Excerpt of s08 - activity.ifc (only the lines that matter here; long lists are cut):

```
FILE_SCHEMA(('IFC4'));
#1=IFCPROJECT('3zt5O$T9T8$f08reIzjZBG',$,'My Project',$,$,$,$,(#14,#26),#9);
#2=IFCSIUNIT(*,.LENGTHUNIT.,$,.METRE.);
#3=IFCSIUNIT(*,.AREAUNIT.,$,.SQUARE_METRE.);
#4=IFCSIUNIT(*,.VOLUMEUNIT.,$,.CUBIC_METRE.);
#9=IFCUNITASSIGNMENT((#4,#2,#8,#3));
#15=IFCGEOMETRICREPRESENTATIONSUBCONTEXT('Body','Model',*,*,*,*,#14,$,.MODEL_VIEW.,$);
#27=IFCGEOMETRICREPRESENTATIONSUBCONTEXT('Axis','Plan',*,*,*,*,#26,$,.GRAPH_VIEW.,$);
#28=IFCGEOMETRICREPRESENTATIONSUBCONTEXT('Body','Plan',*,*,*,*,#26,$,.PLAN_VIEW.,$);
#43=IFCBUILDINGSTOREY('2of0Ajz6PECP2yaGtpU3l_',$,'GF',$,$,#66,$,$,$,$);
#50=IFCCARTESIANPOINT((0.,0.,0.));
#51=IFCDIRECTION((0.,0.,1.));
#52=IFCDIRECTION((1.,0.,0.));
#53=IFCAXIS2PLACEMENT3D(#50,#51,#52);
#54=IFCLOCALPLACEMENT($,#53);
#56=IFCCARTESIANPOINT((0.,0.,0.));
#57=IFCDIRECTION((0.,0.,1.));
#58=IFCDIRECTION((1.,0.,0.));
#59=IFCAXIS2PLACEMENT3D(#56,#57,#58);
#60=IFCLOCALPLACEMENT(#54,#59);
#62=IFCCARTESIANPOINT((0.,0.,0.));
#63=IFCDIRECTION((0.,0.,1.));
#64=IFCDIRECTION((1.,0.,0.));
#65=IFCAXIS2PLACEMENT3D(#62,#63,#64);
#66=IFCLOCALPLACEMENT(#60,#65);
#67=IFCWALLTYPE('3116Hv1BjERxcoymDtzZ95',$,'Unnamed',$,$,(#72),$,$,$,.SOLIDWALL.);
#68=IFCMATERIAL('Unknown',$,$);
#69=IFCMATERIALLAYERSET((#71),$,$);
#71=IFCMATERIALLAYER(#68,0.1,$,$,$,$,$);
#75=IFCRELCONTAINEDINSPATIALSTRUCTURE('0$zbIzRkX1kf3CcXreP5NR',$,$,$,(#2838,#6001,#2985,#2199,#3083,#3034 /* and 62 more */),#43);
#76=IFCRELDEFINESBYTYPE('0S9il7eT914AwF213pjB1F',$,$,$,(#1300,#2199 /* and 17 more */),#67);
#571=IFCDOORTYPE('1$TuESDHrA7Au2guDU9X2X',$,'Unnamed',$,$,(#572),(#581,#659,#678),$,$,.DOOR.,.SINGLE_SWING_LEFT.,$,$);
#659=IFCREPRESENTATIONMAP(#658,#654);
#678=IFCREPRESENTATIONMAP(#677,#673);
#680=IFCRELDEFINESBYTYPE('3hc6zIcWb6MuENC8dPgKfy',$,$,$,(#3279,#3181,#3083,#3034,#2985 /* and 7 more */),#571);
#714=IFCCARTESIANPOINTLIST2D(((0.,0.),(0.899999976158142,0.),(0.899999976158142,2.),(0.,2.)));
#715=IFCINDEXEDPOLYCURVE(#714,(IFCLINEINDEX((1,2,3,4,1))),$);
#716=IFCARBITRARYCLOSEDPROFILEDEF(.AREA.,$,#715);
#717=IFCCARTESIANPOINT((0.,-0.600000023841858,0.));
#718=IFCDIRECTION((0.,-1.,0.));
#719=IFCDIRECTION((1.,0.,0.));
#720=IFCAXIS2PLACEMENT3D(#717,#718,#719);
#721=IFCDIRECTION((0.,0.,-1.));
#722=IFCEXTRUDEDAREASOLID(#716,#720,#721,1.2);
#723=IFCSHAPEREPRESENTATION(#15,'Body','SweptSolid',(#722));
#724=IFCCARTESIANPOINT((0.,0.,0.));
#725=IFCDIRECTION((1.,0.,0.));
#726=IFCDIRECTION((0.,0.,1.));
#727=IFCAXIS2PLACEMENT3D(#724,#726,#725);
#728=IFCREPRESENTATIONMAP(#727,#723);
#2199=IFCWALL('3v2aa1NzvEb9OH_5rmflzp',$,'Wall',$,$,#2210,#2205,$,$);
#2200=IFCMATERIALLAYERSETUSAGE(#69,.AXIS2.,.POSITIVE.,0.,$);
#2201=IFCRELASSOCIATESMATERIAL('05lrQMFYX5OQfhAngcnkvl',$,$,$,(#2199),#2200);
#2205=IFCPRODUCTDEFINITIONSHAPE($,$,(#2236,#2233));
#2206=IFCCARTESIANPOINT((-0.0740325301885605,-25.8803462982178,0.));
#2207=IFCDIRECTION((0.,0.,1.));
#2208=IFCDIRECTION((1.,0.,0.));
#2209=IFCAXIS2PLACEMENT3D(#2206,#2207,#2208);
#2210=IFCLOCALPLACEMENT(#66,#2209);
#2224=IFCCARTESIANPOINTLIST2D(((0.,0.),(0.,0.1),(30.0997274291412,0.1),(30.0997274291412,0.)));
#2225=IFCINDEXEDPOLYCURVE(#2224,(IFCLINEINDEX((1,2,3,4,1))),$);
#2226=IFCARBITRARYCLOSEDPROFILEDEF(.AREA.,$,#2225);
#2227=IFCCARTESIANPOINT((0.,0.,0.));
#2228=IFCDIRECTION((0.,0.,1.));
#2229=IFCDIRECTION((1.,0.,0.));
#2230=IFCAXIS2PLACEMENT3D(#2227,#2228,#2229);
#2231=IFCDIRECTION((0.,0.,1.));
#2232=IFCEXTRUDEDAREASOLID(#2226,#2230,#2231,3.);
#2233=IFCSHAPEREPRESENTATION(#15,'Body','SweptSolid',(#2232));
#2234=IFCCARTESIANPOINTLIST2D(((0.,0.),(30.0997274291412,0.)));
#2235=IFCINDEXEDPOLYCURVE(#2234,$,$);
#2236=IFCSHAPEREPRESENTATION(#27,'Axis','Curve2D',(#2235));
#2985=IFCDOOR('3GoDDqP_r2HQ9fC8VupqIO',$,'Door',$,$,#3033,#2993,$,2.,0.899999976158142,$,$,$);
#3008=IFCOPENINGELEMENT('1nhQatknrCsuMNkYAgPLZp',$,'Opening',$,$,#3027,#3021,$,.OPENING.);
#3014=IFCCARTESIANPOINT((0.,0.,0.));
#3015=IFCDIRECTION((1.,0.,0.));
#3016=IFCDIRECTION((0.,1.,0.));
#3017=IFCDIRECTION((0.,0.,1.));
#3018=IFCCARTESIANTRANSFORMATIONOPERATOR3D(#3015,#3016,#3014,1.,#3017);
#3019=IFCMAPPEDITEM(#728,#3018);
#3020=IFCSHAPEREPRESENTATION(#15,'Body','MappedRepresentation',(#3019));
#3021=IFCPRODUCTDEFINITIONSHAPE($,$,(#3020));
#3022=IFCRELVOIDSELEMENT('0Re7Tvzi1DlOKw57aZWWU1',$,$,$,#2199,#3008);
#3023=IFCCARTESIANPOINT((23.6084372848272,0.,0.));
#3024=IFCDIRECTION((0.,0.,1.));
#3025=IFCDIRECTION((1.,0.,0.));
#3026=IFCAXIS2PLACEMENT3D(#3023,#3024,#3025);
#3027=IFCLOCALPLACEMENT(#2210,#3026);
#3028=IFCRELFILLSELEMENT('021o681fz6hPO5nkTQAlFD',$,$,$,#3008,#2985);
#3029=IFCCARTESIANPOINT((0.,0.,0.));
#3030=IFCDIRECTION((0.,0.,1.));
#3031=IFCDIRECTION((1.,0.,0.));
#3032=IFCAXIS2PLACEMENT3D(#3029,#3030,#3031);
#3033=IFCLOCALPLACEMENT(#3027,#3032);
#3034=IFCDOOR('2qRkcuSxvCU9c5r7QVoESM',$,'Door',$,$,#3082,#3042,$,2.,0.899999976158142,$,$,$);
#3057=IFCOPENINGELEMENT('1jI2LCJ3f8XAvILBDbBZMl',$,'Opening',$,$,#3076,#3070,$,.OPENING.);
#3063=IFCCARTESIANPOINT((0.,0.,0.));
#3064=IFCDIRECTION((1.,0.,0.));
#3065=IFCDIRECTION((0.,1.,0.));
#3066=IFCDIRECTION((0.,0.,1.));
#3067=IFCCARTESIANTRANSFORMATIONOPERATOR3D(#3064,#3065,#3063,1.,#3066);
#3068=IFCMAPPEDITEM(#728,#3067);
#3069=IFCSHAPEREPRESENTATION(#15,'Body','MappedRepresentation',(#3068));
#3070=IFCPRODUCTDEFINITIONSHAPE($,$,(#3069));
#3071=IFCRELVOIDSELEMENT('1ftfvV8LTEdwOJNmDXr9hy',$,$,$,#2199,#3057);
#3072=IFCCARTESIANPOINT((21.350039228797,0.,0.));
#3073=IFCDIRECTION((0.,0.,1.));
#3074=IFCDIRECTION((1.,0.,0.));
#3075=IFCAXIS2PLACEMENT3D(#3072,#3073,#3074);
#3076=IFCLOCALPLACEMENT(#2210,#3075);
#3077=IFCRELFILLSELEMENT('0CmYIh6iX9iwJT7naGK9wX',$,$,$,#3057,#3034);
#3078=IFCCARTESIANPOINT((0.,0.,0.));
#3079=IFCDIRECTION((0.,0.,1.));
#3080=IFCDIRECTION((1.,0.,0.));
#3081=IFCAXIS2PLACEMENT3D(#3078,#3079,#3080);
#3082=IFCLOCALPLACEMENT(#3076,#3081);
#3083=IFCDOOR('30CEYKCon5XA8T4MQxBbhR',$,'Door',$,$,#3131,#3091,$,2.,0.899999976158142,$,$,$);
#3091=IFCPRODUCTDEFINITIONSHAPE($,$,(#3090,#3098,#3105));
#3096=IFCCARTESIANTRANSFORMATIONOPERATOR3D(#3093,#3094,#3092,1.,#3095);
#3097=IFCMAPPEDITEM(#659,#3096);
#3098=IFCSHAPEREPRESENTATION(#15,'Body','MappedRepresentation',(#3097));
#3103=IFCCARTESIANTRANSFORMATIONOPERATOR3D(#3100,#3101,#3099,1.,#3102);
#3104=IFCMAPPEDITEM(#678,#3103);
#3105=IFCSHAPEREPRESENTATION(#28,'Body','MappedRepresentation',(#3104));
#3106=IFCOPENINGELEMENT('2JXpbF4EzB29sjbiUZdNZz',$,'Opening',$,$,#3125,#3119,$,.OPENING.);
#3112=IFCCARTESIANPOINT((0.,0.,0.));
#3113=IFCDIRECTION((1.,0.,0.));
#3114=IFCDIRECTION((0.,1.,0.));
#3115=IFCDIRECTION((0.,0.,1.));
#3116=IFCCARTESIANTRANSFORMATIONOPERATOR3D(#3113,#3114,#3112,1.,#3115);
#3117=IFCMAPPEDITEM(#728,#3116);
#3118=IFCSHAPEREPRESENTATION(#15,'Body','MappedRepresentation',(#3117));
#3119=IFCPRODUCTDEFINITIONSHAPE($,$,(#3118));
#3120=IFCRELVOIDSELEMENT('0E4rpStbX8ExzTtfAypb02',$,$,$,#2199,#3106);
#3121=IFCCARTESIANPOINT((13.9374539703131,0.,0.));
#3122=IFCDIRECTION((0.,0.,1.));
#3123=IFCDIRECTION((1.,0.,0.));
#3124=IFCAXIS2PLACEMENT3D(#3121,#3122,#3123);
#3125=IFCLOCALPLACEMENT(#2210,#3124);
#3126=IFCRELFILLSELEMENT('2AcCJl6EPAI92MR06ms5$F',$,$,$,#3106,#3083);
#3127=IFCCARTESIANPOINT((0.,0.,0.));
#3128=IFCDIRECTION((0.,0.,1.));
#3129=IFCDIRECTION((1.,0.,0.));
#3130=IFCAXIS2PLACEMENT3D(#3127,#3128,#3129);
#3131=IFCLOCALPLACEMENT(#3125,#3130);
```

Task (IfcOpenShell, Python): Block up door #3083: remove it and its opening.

```python
import ifcopenshell
import ifcopenshell.api.feature
import ifcopenshell.api.root
import ifcopenshell.geom
import ifcopenshell.util.shape

model = ifcopenshell.open("s08 - activity.ifc")
settings = ifcopenshell.geom.settings()


def volume(element):
    """Net volume in cubic metres, openings subtracted."""
    shape = ifcopenshell.geom.create_shape(settings, element)
    return ifcopenshell.util.shape.get_volume(shape.geometry)


door = model.by_guid("30CEYKCon5XA8T4MQxBbhR")
opening = door.FillsVoids[0].RelatingOpeningElement
wall = opening.VoidsElements[0].RelatingBuildingElement
before = volume(wall)

ifcopenshell.api.root.remove_product(model, product=door)
ifcopenshell.api.feature.remove_feature(model, feature=opening)

after = volume(wall)

print(f"wall volume {before:.3f} -> {after:.3f} m3")

model.write("s08 - activity_edited.ifc")
```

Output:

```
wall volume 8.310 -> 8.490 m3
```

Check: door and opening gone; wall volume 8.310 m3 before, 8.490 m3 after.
